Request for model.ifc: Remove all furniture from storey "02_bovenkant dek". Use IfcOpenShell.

First a look at what the model holds.

```python
import ifcopenshell
import ifcopenshell.util.element

model = ifcopenshell.open("model.ifc")
print(model.schema)
storey = next(s for s in model.by_type("IfcBuildingStorey") if s.Name == "02_bovenkant dek")
furniture = [e for e in ifcopenshell.util.element.get_decomposition(storey) if e.is_a("IfcFurnishingElement")]
seen = {}
for e in furniture:
    element_type = ifcopenshell.util.element.get_type(e)
    name = element_type.Name if element_type not in (None, e) else None
    seen[name] = seen.get(name, 0) + 1
for name, count in sorted(seen.items(), key=str):
    print(count, "x", name)
```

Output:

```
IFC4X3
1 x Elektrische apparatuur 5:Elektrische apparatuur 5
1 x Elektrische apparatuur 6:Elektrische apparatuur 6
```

```python
import ifcopenshell
import ifcopenshell.api.root
import ifcopenshell.util.element

model = ifcopenshell.open("model.ifc")

storey = next(s for s in model.by_type("IfcBuildingStorey") if s.Name == "02_bovenkant dek")
furniture = [e for e in ifcopenshell.util.element.get_decomposition(storey) if e.is_a("IfcFurnishingElement")]

for e in furniture:
    ifcopenshell.api.root.remove_product(model, product=e)
print(len(furniture), "removed")

model.write("model_updated.ifc")
```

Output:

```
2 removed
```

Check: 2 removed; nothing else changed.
